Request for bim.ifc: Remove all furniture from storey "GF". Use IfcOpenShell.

First a look at what the model holds.

```python
import ifcopenshell
import ifcopenshell.util.element

model = ifcopenshell.open("bim.ifc")
print(model.schema)
storey = next(s for s in model.by_type("IfcBuildingStorey") if s.Name == "GF")
furniture = [e for e in ifcopenshell.util.element.get_decomposition(storey) if e.is_a("IfcFurnishingElement")]
seen = {}
for e in furniture:
    element_type = ifcopenshell.util.element.get_type(e)
    name = element_type.Name if element_type not in (None, e) else None
    seen[name] = seen.get(name, 0) + 1
for name, count in sorted(seen.items(), key=str):
    print(count, "x", name)
```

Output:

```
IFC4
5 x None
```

```python
import ifcopenshell
import ifcopenshell.api.root
import ifcopenshell.util.element

model = ifcopenshell.open("bim.ifc")

storey = next(s for s in model.by_type("IfcBuildingStorey") if s.Name == "GF")
furniture = [e for e in ifcopenshell.util.element.get_decomposition(storey) if e.is_a("IfcFurnishingElement")]

for e in furniture:
    ifcopenshell.api.root.remove_product(model, product=e)
print(len(furniture), "removed")

model.write("bim_rev.ifc")
```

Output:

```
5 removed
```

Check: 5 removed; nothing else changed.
